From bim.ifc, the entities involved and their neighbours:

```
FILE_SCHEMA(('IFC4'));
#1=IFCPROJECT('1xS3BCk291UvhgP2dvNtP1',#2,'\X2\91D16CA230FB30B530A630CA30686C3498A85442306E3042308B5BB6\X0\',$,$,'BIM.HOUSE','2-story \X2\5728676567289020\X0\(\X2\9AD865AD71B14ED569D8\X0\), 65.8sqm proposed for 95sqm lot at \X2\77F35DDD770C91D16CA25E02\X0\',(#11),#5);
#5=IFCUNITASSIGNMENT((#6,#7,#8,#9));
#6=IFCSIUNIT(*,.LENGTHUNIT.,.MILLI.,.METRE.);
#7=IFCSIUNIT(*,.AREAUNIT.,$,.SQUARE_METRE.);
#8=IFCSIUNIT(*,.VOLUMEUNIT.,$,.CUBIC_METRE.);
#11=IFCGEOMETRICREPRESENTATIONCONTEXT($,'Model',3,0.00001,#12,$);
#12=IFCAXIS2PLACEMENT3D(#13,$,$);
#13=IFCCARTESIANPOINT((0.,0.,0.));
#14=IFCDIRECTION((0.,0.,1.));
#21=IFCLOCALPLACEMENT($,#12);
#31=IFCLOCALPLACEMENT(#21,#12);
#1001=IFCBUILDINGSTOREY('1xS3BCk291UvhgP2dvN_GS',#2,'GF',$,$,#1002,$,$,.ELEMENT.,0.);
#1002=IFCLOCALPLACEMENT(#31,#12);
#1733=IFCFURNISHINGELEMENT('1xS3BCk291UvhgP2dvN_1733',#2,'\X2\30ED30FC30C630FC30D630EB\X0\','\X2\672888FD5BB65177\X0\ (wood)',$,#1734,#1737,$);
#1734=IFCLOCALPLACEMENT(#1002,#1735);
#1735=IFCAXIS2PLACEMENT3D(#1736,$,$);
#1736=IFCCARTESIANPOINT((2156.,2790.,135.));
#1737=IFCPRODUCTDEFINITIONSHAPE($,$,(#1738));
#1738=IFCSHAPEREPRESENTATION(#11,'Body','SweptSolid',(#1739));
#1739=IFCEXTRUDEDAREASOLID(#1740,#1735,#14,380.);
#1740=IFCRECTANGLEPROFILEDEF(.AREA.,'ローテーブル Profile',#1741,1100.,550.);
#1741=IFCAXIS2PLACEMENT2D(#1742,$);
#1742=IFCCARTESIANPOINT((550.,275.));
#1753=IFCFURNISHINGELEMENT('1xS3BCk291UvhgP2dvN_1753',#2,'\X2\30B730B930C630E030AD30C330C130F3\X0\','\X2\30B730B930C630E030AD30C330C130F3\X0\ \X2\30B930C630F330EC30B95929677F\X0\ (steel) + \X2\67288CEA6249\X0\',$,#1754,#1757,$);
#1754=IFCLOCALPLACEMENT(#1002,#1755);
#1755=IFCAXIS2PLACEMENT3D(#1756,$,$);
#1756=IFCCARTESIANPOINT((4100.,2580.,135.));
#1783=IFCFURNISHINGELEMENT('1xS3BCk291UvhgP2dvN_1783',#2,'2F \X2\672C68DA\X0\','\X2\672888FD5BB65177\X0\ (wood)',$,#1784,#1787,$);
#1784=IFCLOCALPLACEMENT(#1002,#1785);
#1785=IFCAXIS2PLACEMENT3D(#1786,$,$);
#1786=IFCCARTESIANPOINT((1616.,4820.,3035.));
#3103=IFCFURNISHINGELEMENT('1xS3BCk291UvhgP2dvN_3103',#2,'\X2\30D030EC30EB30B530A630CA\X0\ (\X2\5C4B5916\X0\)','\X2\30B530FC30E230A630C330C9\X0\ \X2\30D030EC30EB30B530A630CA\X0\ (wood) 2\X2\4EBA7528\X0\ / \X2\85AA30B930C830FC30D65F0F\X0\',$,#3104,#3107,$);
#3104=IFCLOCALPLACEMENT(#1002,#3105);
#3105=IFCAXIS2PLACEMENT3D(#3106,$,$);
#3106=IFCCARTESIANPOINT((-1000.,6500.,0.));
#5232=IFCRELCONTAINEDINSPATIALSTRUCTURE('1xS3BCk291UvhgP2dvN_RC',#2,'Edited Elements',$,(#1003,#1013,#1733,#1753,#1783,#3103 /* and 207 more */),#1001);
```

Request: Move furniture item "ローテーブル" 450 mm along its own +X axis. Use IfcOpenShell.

```python
import ifcopenshell
import ifcopenshell.api.geometry
import ifcopenshell.util.placement
import ifcopenshell.util.unit

model = ifcopenshell.open("bim.ifc")
unit_scale = ifcopenshell.util.unit.calculate_unit_scale(model)

item = model.by_id(1733)
matrix = ifcopenshell.util.placement.get_local_placement(item.ObjectPlacement)
matrix[:3, 3] += matrix[:3, 0] * 0.45 / unit_scale
ifcopenshell.api.geometry.edit_object_placement(model, product=item, matrix=matrix, is_si=False)

print(ifcopenshell.util.placement.get_local_placement(item.ObjectPlacement).round(3) + 0.0)

model.write("bim-out.ifc")
```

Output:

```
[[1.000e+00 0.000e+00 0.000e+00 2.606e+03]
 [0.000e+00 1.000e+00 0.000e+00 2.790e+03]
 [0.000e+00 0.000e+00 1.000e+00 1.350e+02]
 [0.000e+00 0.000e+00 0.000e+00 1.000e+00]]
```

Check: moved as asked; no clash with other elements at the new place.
